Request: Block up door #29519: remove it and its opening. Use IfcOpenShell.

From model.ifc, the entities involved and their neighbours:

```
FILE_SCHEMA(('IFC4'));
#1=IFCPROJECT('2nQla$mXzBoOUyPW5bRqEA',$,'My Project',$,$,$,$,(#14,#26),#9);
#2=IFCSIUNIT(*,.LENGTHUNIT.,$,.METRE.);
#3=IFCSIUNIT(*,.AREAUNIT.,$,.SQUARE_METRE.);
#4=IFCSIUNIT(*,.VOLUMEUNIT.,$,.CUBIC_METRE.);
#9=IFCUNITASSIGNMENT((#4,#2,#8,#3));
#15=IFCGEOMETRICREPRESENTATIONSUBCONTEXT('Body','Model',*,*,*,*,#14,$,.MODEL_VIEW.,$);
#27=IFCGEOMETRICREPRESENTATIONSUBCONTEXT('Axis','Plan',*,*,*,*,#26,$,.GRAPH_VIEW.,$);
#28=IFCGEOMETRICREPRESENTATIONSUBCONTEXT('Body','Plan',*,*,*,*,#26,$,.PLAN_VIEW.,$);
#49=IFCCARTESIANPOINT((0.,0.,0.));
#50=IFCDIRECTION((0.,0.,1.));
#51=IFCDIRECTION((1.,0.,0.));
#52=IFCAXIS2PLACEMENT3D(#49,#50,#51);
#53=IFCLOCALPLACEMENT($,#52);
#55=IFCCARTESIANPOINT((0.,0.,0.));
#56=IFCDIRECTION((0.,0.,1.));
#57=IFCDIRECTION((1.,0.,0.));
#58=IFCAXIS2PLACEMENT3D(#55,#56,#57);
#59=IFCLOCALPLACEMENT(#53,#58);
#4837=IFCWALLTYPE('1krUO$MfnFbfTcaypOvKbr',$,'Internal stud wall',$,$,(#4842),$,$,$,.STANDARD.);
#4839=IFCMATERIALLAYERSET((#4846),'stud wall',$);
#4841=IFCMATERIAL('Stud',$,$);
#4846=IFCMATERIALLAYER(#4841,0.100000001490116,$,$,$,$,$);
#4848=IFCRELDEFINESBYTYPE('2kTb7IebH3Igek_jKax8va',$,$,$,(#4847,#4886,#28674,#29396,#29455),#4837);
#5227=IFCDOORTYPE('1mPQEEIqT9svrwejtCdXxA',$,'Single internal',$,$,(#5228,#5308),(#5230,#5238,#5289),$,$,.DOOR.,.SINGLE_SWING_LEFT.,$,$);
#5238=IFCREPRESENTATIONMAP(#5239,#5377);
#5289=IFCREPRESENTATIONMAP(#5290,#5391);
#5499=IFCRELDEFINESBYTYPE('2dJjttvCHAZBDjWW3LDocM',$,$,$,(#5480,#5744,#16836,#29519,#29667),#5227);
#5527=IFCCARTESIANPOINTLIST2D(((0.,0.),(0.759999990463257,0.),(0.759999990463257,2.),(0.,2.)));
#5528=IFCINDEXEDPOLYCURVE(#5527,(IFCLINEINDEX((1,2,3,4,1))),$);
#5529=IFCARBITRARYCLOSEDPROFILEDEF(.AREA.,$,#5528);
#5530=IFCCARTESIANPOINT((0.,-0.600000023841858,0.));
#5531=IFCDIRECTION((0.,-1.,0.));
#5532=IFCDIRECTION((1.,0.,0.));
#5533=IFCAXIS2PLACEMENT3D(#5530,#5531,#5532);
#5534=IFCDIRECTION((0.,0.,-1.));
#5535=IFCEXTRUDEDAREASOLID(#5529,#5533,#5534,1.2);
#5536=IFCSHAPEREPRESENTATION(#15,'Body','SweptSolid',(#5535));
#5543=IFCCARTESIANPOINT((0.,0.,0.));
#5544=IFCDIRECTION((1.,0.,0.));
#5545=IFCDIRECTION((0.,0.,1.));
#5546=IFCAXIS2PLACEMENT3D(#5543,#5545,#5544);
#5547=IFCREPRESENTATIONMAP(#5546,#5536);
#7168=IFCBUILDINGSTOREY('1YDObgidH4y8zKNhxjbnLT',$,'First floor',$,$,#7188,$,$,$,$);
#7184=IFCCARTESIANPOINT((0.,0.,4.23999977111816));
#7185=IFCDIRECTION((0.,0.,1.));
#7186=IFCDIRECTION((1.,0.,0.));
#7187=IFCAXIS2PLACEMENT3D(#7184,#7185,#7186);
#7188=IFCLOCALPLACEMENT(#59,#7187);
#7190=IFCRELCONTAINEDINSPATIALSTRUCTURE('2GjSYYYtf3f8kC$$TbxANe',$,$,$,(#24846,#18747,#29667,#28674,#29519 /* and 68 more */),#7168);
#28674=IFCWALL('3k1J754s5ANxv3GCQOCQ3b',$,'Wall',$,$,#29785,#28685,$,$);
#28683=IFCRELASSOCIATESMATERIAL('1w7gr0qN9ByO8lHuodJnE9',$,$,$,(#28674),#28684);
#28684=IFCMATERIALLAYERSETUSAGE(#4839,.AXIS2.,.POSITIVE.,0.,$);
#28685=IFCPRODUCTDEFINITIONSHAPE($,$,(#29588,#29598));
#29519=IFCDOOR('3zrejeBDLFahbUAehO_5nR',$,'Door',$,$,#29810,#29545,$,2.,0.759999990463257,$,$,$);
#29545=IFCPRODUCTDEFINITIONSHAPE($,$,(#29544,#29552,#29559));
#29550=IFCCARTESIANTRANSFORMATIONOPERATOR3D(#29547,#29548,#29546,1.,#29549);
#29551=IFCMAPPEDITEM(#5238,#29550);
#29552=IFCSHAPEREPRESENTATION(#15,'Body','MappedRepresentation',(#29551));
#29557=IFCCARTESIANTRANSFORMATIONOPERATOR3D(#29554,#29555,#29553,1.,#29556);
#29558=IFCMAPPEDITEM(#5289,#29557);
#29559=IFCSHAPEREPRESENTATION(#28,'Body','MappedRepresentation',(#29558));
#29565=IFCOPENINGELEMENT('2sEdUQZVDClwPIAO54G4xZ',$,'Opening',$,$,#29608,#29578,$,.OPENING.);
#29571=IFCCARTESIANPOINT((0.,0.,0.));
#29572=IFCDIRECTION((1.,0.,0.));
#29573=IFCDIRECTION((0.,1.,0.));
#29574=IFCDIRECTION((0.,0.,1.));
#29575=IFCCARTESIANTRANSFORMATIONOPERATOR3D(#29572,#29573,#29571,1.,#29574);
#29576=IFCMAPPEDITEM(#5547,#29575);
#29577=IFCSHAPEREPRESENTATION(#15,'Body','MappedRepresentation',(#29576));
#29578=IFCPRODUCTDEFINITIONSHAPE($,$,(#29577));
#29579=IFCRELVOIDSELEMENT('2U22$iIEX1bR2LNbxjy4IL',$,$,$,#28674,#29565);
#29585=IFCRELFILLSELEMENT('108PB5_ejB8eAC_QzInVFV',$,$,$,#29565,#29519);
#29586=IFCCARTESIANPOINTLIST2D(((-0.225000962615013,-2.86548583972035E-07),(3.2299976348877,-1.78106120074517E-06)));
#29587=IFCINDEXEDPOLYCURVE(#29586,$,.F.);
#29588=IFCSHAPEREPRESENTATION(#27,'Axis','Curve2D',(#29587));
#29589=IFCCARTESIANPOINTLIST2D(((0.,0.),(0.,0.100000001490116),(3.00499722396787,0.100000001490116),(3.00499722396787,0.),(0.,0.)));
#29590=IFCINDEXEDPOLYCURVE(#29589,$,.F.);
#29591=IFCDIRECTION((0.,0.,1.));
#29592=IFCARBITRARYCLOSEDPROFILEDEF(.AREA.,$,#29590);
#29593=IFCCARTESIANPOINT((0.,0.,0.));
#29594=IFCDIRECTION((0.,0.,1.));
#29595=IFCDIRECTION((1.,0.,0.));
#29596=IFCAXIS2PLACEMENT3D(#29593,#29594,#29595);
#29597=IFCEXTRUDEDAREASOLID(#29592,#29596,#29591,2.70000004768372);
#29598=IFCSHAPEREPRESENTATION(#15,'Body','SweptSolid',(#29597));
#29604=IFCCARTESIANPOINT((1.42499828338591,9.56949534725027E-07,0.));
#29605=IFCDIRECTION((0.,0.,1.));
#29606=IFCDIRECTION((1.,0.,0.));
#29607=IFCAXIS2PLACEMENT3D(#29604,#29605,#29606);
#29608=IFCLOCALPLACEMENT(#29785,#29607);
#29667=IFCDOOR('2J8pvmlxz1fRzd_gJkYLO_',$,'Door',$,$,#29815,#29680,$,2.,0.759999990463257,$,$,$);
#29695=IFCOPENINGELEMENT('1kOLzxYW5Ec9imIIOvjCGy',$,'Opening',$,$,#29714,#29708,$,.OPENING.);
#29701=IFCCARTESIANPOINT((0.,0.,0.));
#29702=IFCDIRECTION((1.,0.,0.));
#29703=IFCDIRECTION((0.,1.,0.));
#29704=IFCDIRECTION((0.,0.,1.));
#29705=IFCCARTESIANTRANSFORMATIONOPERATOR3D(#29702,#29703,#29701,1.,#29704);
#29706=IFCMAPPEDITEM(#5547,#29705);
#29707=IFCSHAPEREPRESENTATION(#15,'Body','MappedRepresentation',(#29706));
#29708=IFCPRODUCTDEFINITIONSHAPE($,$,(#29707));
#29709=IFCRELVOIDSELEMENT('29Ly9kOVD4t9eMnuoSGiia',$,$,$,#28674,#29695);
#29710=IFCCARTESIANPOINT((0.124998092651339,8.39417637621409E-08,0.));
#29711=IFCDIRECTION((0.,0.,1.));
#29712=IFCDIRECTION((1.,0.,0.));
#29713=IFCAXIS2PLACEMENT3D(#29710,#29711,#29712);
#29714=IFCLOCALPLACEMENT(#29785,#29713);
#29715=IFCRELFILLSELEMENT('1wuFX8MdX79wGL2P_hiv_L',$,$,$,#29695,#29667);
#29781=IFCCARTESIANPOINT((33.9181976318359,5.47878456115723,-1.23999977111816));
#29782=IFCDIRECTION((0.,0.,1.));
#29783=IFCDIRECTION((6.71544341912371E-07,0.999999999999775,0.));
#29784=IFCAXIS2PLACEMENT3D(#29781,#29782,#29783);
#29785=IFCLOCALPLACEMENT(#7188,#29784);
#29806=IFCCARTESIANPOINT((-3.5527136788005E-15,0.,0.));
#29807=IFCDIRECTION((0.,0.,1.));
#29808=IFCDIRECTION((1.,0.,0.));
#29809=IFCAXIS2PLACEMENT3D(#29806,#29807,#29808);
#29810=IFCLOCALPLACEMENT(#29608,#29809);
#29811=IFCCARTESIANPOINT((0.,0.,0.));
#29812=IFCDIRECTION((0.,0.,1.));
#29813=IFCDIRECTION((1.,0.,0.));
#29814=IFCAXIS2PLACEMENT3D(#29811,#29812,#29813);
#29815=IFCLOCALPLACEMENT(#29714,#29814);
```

```python
import ifcopenshell
import ifcopenshell.api.feature
import ifcopenshell.api.root
import ifcopenshell.geom
import ifcopenshell.util.shape

model = ifcopenshell.open("model.ifc")
settings = ifcopenshell.geom.settings()


def volume(element):
    """Net volume in cubic metres, openings subtracted."""
    shape = ifcopenshell.geom.create_shape(settings, element)
    return ifcopenshell.util.shape.get_volume(shape.geometry)


door = model.by_id(29519)
opening = door.FillsVoids[0].RelatingOpeningElement
wall = opening.VoidsElements[0].RelatingBuildingElement
before = volume(wall)

ifcopenshell.api.root.remove_product(model, product=door)
ifcopenshell.api.feature.remove_feature(model, feature=opening)

after = volume(wall)

print(f"wall volume {before:.3f} -> {after:.3f} m3")

model.write("model_updated.ifc")
```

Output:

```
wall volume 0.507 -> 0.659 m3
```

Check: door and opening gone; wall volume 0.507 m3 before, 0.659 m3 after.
